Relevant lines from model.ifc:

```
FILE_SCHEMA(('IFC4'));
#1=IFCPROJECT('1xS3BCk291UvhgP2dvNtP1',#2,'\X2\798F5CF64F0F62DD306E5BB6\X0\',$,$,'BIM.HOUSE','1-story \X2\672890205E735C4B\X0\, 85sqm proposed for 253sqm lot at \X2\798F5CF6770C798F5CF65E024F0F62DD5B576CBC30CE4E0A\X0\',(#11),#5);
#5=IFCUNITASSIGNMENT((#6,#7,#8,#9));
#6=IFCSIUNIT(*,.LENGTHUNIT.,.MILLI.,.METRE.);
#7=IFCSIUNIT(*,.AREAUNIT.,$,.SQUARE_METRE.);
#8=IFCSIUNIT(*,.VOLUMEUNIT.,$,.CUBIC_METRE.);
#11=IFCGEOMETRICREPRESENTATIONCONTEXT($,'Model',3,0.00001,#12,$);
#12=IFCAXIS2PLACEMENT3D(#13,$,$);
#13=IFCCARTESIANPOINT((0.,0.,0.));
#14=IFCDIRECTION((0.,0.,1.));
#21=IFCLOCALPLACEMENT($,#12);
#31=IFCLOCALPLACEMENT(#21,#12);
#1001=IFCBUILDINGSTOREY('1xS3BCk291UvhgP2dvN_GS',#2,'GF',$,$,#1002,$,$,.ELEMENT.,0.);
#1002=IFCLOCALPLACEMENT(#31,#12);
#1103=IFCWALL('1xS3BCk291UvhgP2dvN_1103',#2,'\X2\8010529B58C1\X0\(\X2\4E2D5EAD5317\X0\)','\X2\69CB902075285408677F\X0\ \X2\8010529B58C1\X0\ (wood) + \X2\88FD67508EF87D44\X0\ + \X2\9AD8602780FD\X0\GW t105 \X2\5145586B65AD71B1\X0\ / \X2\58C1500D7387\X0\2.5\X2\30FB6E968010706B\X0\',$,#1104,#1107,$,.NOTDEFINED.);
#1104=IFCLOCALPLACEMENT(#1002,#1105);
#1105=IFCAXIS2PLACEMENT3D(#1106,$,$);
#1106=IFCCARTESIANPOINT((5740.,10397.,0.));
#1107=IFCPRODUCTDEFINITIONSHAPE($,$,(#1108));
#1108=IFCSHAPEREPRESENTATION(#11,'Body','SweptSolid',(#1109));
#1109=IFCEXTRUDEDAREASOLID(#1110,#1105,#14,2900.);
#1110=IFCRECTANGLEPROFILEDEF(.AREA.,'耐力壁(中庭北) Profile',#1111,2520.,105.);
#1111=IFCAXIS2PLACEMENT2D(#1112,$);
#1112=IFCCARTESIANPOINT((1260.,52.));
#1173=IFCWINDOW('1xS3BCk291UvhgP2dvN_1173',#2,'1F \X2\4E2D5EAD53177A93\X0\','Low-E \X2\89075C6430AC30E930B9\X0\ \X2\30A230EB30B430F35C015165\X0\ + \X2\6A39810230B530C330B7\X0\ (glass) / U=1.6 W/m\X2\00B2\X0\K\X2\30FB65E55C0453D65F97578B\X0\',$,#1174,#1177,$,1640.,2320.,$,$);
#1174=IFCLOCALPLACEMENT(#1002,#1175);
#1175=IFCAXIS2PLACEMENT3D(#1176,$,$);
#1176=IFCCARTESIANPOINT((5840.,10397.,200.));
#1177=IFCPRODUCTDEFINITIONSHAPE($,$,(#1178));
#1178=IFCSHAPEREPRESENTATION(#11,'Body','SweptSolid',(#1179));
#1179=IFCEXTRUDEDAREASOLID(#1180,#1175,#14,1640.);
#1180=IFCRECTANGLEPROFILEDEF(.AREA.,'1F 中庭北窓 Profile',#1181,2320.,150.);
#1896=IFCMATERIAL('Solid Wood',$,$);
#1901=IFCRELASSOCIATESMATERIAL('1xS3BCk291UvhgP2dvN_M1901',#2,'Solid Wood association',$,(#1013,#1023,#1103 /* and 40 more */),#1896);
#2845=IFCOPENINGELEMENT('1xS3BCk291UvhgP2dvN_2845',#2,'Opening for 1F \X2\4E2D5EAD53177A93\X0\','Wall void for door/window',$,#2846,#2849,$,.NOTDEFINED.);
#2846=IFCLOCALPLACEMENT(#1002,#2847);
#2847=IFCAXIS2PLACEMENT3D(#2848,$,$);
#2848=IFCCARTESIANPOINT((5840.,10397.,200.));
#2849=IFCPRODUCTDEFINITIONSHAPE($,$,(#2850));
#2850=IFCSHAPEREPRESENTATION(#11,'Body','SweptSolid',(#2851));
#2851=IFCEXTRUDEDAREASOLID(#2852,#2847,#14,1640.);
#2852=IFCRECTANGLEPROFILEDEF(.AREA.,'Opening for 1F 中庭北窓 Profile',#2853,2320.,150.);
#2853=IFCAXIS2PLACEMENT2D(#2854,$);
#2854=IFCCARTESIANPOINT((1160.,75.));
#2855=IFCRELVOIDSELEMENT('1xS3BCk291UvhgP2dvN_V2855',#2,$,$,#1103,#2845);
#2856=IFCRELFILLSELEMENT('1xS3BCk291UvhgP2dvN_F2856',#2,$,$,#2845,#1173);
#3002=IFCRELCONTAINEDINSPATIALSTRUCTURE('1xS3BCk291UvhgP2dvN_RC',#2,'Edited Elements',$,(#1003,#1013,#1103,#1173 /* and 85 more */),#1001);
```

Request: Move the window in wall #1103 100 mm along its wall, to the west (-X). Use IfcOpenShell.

```python
import ifcopenshell
import ifcopenshell.api.geometry
import ifcopenshell.util.placement
import ifcopenshell.util.unit

model = ifcopenshell.open("model.ifc")
unit_scale = ifcopenshell.util.unit.calculate_unit_scale(model)

window = model.by_guid("1xS3BCk291UvhgP2dvN_1173")
opening = window.FillsVoids[0].RelatingOpeningElement
wall = opening.VoidsElements[0].RelatingBuildingElement

wall_matrix = ifcopenshell.util.placement.get_local_placement(wall.ObjectPlacement)
shift = wall_matrix[:3, 0] * -0.1 / unit_scale
before = ifcopenshell.util.placement.get_local_placement(window.ObjectPlacement)[:3, 3].copy()

# The window is not placed relative to its opening, so move both.
for product in (opening, window):
    matrix = ifcopenshell.util.placement.get_local_placement(product.ObjectPlacement)
    matrix[:3, 3] += shift
    ifcopenshell.api.geometry.edit_object_placement(model, product=product, matrix=matrix, is_si=False)

after = ifcopenshell.util.placement.get_local_placement(window.ObjectPlacement)[:3, 3]
print("window moved by", (after - before).round(3) + 0.0)

model.write("model_updated.ifc")
```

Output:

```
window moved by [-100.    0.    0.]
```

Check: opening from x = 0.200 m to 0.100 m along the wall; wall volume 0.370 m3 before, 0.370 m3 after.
